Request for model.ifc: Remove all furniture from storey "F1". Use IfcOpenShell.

First a look at what the model holds.

```python
import ifcopenshell
import ifcopenshell.util.element

model = ifcopenshell.open("model.ifc")
print(model.schema)
storey = next(s for s in model.by_type("IfcBuildingStorey") if s.Name == "F1")
furniture = [e for e in ifcopenshell.util.element.get_decomposition(storey) if e.is_a("IfcFurnishingElement")]
seen = {}
for e in furniture:
    element_type = ifcopenshell.util.element.get_type(e)
    name = element_type.Name if element_type not in (None, e) else None
    seen[name] = seen.get(name, 0) + 1
for name, count in sorted(seen.items(), key=str):
    print(count, "x", name)
```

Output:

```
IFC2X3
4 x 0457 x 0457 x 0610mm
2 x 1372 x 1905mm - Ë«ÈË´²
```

```python
import ifcopenshell
import ifcopenshell.api.root
import ifcopenshell.util.element

model = ifcopenshell.open("model.ifc")

storey = next(s for s in model.by_type("IfcBuildingStorey") if s.Name == "F1")
furniture = [e for e in ifcopenshell.util.element.get_decomposition(storey) if e.is_a("IfcFurnishingElement")]

for e in furniture:
    ifcopenshell.api.root.remove_product(model, product=e)
print(len(furniture), "removed")

model.write("model_edited.ifc")
```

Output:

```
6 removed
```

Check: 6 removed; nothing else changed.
